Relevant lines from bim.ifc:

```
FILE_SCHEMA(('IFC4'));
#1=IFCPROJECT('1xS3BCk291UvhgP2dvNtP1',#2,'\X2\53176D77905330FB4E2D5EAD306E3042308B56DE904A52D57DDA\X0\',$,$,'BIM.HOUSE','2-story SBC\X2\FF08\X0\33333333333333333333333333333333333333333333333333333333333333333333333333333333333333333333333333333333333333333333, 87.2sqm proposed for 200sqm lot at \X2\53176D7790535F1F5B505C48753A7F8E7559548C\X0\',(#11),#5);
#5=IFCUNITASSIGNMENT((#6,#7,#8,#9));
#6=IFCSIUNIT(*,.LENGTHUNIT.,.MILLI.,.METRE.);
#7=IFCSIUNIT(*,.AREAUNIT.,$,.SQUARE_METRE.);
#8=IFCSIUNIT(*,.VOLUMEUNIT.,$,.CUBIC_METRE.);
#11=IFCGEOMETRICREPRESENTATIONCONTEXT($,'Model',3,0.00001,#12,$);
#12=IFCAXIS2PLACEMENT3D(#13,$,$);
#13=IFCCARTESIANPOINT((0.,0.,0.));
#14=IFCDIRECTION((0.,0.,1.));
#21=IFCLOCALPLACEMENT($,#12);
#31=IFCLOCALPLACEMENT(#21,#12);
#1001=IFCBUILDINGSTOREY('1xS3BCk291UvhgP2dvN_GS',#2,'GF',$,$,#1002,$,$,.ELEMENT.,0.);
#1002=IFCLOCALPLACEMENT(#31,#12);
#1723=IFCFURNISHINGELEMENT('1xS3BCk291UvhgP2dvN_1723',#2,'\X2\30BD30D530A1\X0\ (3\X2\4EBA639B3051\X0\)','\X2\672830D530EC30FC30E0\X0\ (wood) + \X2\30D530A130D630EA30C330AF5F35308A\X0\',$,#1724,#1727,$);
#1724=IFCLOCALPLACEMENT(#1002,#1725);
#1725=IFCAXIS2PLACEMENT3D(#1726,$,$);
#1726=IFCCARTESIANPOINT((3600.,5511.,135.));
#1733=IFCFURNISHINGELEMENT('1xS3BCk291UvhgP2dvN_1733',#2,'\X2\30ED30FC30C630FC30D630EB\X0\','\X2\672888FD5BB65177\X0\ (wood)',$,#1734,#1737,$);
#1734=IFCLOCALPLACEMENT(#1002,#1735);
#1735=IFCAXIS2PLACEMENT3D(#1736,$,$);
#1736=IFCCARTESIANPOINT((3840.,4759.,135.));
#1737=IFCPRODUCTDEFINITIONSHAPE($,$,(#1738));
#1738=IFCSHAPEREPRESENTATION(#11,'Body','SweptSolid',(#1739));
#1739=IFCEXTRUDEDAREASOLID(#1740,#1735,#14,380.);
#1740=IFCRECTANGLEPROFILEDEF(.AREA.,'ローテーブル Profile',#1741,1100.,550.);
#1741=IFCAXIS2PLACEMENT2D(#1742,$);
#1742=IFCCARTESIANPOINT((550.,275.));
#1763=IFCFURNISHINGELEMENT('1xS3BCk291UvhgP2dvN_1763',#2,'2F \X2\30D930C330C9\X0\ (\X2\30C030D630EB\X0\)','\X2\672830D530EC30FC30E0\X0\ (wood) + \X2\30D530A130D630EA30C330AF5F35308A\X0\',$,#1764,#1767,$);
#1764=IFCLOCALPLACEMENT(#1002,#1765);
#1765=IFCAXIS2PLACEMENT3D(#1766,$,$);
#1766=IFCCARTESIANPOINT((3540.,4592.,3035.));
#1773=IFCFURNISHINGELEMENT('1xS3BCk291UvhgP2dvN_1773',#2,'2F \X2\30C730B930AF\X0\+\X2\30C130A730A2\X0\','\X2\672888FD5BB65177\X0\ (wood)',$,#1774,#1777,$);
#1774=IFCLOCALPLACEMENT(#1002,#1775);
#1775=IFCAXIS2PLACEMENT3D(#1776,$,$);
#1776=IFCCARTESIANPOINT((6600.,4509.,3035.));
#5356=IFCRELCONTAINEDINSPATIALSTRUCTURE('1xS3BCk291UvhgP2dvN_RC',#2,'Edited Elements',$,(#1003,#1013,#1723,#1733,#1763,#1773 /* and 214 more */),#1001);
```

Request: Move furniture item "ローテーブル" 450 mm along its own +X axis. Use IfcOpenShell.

```python
import ifcopenshell
import ifcopenshell.api.geometry
import ifcopenshell.util.placement

model = ifcopenshell.open("bim.ifc")

item = model.by_guid("1xS3BCk291UvhgP2dvN_1733")
matrix = ifcopenshell.util.placement.get_local_placement(item.ObjectPlacement)
matrix[:3, 3] += matrix[:3, 0] * 450.0
ifcopenshell.api.geometry.edit_object_placement(model, product=item, matrix=matrix, is_si=False)

print(ifcopenshell.util.placement.get_local_placement(item.ObjectPlacement).round(3) + 0.0)

model.write("bim_updated.ifc")
```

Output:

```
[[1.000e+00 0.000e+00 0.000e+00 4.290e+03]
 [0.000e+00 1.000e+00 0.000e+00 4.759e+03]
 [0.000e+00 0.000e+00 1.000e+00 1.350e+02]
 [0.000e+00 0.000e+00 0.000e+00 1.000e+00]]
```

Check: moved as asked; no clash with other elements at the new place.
